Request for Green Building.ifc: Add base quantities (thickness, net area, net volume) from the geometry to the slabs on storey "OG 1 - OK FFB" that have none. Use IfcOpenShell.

First a look at what the model holds.

```python
import ifcopenshell
import ifcopenshell.util.element
import ifcopenshell.util.unit

model = ifcopenshell.open("Green Building.ifc")
print(model.schema)
for unit_type in ("LENGTHUNIT", "AREAUNIT", "VOLUMEUNIT"):
    print(unit_type, ifcopenshell.util.unit.calculate_unit_scale(model, unit_type))
storey = next(s for s in model.by_type("IfcBuildingStorey") if s.Name == "OG 1 - OK FFB")
slabs = [e for e in ifcopenshell.util.element.get_decomposition(storey) if e.is_a("IfcSlab")]
for e in sorted(slabs, key=lambda e: e.id()):
    print(e.id(), e.is_a(), e.Name, list(ifcopenshell.util.element.get_psets(e, qtos_only=True)), sep=" | ")
```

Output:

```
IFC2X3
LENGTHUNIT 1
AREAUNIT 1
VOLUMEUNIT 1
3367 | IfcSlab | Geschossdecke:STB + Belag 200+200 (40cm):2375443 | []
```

```python
import ifcopenshell
import ifcopenshell.api.pset
import ifcopenshell.geom
import ifcopenshell.util.element
import ifcopenshell.util.shape
import ifcopenshell.util.unit

model = ifcopenshell.open("Green Building.ifc")
unit_scale = ifcopenshell.util.unit.calculate_unit_scale(model)
area_scale = ifcopenshell.util.unit.calculate_unit_scale(model, "AREAUNIT")
volume_scale = ifcopenshell.util.unit.calculate_unit_scale(model, "VOLUMEUNIT")
settings = ifcopenshell.geom.settings()

storey = next(s for s in model.by_type("IfcBuildingStorey") if s.Name == "OG 1 - OK FFB")
slabs = [e for e in ifcopenshell.util.element.get_decomposition(storey) if e.is_a("IfcSlab")]

for e in sorted(slabs, key=lambda e: e.id()):
    if ifcopenshell.util.element.get_psets(e, qtos_only=True, should_inherit=False):
        continue
    # Geometry comes back in metres, in the element's own axes.
    shape = ifcopenshell.geom.create_shape(settings, e)
    values = {
        "Width": ifcopenshell.util.shape.get_z(shape.geometry) / unit_scale,
        "NetArea": ifcopenshell.util.shape.get_footprint_area(shape.geometry) / area_scale,
        "NetVolume": ifcopenshell.util.shape.get_volume(shape.geometry) / volume_scale,
    }
    qto = ifcopenshell.api.pset.add_qto(model, product=e, name="BaseQuantities")
    ifcopenshell.api.pset.edit_qto(model, qto=qto, properties=values)
    print(e.id(), {k: round(v, 3) for k, v in values.items()})

model.write("Green Building_edited.ifc")
```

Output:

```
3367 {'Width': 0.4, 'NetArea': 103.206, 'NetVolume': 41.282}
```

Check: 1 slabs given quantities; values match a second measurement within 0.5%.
